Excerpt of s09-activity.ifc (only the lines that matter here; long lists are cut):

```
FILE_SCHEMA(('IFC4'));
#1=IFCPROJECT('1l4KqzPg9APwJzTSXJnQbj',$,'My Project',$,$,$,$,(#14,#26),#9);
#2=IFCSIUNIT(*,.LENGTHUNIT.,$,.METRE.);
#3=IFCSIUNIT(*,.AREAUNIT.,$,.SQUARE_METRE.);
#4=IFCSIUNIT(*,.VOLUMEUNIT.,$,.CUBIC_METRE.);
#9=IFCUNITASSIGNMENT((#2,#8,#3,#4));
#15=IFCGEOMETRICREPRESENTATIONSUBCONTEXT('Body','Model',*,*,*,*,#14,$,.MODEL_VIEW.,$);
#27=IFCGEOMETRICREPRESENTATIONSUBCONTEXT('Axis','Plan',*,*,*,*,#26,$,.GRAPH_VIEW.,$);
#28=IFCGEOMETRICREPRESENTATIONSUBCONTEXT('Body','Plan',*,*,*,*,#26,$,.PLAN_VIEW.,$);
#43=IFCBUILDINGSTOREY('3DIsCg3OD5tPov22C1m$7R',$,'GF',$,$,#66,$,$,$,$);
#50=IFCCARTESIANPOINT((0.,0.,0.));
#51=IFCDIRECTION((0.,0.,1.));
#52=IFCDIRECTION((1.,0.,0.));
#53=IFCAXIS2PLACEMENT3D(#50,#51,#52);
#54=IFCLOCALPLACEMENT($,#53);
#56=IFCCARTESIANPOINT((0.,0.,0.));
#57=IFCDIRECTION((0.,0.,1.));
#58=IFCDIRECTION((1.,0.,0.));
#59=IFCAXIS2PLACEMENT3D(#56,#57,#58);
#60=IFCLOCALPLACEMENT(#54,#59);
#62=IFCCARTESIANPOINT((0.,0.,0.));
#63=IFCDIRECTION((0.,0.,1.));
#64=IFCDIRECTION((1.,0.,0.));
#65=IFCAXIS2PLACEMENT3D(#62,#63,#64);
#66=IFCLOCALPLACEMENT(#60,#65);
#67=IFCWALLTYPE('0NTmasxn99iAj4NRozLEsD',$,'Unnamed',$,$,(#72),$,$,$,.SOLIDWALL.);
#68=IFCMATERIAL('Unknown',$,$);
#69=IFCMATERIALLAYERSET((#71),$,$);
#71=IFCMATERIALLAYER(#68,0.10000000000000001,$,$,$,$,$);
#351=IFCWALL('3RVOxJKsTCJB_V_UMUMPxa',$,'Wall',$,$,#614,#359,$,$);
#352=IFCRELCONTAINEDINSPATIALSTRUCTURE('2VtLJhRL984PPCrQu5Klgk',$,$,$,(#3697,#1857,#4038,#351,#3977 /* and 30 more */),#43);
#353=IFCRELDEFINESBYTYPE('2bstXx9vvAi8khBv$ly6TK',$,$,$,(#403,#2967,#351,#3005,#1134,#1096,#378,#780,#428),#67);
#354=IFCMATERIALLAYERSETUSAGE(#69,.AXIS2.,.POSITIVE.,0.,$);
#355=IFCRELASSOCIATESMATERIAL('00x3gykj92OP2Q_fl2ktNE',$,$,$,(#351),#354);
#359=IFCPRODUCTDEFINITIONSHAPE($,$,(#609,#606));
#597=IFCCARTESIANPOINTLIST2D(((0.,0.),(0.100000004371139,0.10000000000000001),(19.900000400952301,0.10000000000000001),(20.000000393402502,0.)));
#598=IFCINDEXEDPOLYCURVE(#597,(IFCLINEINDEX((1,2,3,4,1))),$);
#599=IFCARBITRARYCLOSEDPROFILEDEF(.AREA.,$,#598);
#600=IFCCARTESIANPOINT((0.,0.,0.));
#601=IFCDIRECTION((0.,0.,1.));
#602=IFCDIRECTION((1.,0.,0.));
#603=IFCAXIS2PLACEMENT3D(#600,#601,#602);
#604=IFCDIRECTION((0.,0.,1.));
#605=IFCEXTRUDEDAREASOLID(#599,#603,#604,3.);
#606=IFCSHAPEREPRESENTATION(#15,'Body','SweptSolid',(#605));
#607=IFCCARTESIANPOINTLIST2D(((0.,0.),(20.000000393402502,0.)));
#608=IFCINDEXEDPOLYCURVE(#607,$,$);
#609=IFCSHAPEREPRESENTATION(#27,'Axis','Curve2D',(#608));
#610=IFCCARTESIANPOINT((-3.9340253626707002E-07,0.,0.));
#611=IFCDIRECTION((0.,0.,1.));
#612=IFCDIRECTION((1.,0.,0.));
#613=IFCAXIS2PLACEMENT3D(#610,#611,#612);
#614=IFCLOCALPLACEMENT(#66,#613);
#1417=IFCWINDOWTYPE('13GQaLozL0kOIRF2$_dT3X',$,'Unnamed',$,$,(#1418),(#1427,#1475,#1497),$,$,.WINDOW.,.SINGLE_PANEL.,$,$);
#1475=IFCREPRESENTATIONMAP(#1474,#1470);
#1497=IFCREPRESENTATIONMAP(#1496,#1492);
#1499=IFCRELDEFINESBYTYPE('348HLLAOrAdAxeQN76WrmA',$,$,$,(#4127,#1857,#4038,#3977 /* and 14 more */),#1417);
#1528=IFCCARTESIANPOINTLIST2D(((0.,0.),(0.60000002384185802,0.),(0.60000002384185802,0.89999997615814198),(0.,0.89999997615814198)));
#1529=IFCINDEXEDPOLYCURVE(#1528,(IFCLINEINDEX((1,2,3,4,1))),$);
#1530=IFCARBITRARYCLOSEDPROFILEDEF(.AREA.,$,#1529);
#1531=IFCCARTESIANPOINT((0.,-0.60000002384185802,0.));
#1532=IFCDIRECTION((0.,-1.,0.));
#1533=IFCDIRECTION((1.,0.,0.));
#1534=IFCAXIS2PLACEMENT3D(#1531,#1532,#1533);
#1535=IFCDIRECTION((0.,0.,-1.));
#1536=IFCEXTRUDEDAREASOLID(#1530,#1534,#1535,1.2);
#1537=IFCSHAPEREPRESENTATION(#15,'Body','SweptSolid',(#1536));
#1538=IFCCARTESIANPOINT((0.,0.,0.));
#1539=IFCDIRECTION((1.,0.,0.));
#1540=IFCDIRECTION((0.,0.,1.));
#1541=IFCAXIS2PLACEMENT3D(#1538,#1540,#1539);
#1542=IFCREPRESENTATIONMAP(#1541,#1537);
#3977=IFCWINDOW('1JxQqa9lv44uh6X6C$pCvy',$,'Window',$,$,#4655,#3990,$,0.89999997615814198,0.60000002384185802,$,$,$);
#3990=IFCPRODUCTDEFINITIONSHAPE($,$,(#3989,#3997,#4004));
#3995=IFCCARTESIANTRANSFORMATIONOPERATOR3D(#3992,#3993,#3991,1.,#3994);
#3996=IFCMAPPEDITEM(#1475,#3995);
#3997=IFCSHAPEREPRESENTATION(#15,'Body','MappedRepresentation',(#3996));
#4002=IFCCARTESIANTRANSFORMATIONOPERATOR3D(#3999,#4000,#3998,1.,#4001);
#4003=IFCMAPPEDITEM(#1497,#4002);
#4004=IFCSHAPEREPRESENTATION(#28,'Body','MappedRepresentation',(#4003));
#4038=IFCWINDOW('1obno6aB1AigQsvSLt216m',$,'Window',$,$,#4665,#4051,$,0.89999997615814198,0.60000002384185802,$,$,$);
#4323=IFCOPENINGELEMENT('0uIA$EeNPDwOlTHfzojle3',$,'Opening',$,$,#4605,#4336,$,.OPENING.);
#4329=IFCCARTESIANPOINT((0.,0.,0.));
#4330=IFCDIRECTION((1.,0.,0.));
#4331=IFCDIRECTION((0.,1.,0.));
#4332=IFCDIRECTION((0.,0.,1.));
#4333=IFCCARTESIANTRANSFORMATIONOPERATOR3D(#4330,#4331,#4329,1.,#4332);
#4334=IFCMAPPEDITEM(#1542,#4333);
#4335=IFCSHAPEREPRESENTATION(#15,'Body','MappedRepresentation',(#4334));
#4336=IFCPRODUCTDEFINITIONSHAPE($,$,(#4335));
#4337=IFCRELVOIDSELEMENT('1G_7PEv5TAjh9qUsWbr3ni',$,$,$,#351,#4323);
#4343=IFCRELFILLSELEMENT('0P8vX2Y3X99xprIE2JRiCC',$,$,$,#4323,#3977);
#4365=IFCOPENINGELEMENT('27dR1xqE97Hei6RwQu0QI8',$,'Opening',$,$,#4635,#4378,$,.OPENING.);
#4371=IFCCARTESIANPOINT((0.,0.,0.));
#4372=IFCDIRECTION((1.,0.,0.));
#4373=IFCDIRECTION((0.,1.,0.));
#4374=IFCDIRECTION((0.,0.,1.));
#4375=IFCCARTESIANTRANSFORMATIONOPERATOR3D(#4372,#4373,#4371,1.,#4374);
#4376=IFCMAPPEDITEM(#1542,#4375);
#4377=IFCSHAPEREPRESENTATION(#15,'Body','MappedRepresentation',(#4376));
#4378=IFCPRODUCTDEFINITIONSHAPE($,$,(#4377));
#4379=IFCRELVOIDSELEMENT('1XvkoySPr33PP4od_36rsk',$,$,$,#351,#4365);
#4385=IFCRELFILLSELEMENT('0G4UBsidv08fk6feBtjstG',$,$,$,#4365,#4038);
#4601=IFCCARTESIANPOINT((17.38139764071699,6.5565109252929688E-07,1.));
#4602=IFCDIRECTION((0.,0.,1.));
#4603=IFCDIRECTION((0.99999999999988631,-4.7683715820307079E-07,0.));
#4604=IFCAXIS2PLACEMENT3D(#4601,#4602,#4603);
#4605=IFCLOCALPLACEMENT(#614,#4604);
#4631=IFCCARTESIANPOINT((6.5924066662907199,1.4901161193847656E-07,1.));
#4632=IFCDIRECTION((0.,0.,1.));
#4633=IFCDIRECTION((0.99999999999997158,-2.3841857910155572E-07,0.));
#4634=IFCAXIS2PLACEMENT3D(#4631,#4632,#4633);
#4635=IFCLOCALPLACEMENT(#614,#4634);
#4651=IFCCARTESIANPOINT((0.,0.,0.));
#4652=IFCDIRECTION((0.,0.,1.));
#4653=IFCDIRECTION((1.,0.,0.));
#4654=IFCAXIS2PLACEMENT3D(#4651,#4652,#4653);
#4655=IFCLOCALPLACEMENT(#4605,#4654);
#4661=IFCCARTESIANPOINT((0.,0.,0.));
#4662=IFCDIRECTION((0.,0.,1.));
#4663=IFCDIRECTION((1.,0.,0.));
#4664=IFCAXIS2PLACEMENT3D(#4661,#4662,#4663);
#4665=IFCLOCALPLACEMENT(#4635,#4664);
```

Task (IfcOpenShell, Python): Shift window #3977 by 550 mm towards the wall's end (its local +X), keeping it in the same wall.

```python
import ifcopenshell
import ifcopenshell.api.geometry
import ifcopenshell.util.placement

model = ifcopenshell.open("s09-activity.ifc")

window = model.by_guid("1JxQqa9lv44uh6X6C$pCvy")
opening = window.FillsVoids[0].RelatingOpeningElement
wall = opening.VoidsElements[0].RelatingBuildingElement

wall_matrix = ifcopenshell.util.placement.get_local_placement(wall.ObjectPlacement)
shift = wall_matrix[:3, 0] * 0.55
before = ifcopenshell.util.placement.get_local_placement(window.ObjectPlacement)[:3, 3].copy()

# The window is placed relative to its opening, so it follows when the opening moves.
matrix = ifcopenshell.util.placement.get_local_placement(opening.ObjectPlacement)
matrix[:3, 3] += shift
ifcopenshell.api.geometry.edit_object_placement(
    model, product=opening, matrix=matrix, is_si=False, should_transform_children=True
)

after = ifcopenshell.util.placement.get_local_placement(window.ObjectPlacement)[:3, 3]
print("window moved by", (after - before).round(3) + 0.0)

model.write("s09-activity_edited.ifc")
```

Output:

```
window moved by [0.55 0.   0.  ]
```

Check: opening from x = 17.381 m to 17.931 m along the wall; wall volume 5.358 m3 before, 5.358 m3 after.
